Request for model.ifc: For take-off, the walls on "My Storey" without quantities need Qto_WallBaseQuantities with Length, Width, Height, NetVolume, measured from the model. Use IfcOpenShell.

First a look at what the model holds.

```python
import ifcopenshell
import ifcopenshell.util.element
import ifcopenshell.util.unit

model = ifcopenshell.open("model.ifc")
print(model.schema)
for unit_type in ("LENGTHUNIT", "AREAUNIT", "VOLUMEUNIT"):
    print(unit_type, ifcopenshell.util.unit.calculate_unit_scale(model, unit_type))
storey = next(s for s in model.by_type("IfcBuildingStorey") if s.Name == "My Storey")
walls = [e for e in ifcopenshell.util.element.get_decomposition(storey) if e.is_a("IfcWall")]
for e in sorted(walls, key=lambda e: e.id()):
    print(e.id(), e.is_a(), e.Name, list(ifcopenshell.util.element.get_psets(e, qtos_only=True)), sep=" | ")
```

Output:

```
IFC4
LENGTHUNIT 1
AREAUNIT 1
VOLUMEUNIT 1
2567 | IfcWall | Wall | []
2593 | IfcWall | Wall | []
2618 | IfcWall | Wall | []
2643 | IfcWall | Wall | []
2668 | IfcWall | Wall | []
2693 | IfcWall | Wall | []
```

```python
import ifcopenshell
import ifcopenshell.api.pset
import ifcopenshell.geom
import ifcopenshell.util.element
import ifcopenshell.util.shape
import ifcopenshell.util.unit

model = ifcopenshell.open("model.ifc")
unit_scale = ifcopenshell.util.unit.calculate_unit_scale(model)
volume_scale = ifcopenshell.util.unit.calculate_unit_scale(model, "VOLUMEUNIT")
settings = ifcopenshell.geom.settings()

storey = next(s for s in model.by_type("IfcBuildingStorey") if s.Name == "My Storey")
walls = [e for e in ifcopenshell.util.element.get_decomposition(storey) if e.is_a("IfcWall")]

for e in sorted(walls, key=lambda e: e.id()):
    if ifcopenshell.util.element.get_psets(e, qtos_only=True, should_inherit=False):
        continue
    # Geometry comes back in metres, in the element's own axes.
    shape = ifcopenshell.geom.create_shape(settings, e)
    values = {
        "Length": ifcopenshell.util.shape.get_x(shape.geometry) / unit_scale,
        "Width": ifcopenshell.util.shape.get_y(shape.geometry) / unit_scale,
        "Height": ifcopenshell.util.shape.get_z(shape.geometry) / unit_scale,
        "NetVolume": ifcopenshell.util.shape.get_volume(shape.geometry) / volume_scale,
    }
    qto = ifcopenshell.api.pset.add_qto(model, product=e, name="Qto_WallBaseQuantities")
    ifcopenshell.api.pset.edit_qto(model, qto=qto, properties=values)
    print(e.id(), {k: round(v, 3) for k, v in values.items()})

model.write("model_rev.ifc")
```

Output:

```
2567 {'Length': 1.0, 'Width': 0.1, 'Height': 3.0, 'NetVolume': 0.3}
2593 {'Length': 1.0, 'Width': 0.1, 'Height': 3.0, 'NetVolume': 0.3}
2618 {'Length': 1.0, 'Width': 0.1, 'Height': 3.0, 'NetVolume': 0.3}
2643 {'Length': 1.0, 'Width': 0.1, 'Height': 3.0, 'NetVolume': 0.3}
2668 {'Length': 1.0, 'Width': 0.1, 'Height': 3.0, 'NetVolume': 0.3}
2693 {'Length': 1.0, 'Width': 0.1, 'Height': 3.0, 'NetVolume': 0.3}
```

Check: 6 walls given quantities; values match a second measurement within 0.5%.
